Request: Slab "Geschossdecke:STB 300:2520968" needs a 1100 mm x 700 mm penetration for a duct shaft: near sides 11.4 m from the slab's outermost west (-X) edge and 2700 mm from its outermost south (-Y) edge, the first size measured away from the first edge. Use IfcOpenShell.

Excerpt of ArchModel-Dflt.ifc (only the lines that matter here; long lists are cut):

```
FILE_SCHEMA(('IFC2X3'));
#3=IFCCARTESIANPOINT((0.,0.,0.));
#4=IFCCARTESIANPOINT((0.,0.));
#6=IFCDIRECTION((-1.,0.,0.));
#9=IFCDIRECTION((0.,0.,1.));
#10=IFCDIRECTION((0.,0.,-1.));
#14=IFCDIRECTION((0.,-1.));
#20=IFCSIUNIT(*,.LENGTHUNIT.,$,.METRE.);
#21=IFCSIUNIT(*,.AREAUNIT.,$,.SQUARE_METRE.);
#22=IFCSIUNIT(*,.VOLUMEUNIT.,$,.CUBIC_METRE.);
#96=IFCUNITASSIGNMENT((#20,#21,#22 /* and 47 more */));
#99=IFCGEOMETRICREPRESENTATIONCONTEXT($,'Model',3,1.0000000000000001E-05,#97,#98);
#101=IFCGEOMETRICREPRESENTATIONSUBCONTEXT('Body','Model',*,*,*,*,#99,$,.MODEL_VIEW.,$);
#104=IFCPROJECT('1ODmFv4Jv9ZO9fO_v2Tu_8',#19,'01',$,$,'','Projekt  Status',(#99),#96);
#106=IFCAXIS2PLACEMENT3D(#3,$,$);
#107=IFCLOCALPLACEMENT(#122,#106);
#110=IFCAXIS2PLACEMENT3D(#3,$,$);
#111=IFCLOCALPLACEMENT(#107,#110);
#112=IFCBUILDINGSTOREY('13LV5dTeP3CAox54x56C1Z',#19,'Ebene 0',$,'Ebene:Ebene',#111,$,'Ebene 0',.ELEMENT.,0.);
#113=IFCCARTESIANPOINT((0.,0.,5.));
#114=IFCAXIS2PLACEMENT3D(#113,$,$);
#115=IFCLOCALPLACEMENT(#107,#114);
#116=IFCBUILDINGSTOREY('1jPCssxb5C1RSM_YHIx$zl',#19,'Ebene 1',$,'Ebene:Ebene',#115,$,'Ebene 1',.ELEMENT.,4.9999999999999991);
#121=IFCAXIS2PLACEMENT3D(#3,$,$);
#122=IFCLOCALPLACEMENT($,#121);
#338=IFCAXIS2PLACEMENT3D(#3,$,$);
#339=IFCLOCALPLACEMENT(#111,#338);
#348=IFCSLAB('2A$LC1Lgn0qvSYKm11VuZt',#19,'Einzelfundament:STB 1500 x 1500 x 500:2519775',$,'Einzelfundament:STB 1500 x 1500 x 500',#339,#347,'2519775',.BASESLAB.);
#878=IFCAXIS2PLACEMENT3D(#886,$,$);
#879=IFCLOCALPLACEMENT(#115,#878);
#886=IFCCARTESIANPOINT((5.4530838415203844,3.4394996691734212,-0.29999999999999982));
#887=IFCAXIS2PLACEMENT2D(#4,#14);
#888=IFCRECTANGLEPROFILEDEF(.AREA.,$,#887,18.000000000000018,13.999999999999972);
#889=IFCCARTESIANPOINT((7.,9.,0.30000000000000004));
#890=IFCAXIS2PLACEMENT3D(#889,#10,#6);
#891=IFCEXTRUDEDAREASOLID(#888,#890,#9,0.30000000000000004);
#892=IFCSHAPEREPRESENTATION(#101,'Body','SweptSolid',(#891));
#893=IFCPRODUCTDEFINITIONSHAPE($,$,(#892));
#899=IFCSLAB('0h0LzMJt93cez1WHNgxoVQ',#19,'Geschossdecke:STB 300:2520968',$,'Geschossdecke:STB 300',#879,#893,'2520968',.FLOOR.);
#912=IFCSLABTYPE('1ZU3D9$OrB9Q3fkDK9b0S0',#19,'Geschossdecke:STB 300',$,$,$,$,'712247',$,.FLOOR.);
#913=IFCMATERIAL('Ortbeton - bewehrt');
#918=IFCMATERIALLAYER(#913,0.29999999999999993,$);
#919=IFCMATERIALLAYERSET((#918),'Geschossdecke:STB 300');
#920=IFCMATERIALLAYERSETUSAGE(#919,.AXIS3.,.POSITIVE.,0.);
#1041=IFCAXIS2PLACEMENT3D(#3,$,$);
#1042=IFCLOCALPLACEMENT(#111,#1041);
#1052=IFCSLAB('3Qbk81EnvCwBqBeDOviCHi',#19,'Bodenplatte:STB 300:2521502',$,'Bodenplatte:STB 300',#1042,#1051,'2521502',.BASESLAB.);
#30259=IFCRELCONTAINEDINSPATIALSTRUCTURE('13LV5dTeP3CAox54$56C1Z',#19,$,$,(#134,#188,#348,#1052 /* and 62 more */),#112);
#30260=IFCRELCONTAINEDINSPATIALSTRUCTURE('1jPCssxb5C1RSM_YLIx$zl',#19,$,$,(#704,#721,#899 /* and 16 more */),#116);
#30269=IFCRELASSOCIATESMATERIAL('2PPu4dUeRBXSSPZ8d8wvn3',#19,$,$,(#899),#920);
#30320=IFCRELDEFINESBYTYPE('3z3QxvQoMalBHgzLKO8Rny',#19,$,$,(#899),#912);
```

```python
import numpy as np
import ifcopenshell
import ifcopenshell.api.feature
import ifcopenshell.api.geometry
import ifcopenshell.api.root
import ifcopenshell.geom
import ifcopenshell.util.placement
import ifcopenshell.util.representation
import ifcopenshell.util.shape
import ifcopenshell.util.unit

model = ifcopenshell.open("ArchModel-Dflt.ifc")
unit_scale = ifcopenshell.util.unit.calculate_unit_scale(model)
settings = ifcopenshell.geom.settings()


def volume(element):
    """Net volume in cubic metres, openings subtracted."""
    shape = ifcopenshell.geom.create_shape(settings, element)
    return ifcopenshell.util.shape.get_volume(shape.geometry)


slab = model.by_guid("0h0LzMJt93cez1WHNgxoVQ")
before = volume(slab)

# Extent in the slab's own axes, in metres. The edges named are its -X and -Y sides.
slab_shape = ifcopenshell.geom.create_shape(settings, slab)
vertices = ifcopenshell.util.shape.get_vertices(slab_shape.geometry)
x_min, y_min, bottom = vertices.min(axis=0)
top = vertices[:, 2].max()

opening = ifcopenshell.api.root.create_entity(model, ifc_class="IfcOpeningElement", name="Duct shaft opening")
context = ifcopenshell.util.representation.get_context(model, "Model", "Body", "MODEL_VIEW")
width, depth = 1.1, 0.7
outline = [(0.0, 0.0), (width, 0.0), (width, depth), (0.0, depth), (0.0, 0.0)]
# Overshoot both faces by 50 mm so the cut is clean.
shape = ifcopenshell.api.geometry.add_slab_representation(
    model, context=context, depth=top - bottom + 0.1, polyline=outline
)
ifcopenshell.api.geometry.assign_representation(model, product=opening, representation=shape)

matrix = ifcopenshell.util.placement.get_local_placement(slab.ObjectPlacement)
matrix[:, 3] = matrix @ np.append(np.array([x_min + 11.4, y_min + 2.7, bottom - 0.05]) / unit_scale, 1.0)
ifcopenshell.api.geometry.edit_object_placement(model, product=opening, matrix=matrix, is_si=False)
ifcopenshell.api.feature.add_feature(model, feature=opening, element=slab)

after = volume(slab)

print(f"slab volume {before:.3f} -> {after:.3f} m3")

model.write("ArchModel-Dflt_updated.ifc")
```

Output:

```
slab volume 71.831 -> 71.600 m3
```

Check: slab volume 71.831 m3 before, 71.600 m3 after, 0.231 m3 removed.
